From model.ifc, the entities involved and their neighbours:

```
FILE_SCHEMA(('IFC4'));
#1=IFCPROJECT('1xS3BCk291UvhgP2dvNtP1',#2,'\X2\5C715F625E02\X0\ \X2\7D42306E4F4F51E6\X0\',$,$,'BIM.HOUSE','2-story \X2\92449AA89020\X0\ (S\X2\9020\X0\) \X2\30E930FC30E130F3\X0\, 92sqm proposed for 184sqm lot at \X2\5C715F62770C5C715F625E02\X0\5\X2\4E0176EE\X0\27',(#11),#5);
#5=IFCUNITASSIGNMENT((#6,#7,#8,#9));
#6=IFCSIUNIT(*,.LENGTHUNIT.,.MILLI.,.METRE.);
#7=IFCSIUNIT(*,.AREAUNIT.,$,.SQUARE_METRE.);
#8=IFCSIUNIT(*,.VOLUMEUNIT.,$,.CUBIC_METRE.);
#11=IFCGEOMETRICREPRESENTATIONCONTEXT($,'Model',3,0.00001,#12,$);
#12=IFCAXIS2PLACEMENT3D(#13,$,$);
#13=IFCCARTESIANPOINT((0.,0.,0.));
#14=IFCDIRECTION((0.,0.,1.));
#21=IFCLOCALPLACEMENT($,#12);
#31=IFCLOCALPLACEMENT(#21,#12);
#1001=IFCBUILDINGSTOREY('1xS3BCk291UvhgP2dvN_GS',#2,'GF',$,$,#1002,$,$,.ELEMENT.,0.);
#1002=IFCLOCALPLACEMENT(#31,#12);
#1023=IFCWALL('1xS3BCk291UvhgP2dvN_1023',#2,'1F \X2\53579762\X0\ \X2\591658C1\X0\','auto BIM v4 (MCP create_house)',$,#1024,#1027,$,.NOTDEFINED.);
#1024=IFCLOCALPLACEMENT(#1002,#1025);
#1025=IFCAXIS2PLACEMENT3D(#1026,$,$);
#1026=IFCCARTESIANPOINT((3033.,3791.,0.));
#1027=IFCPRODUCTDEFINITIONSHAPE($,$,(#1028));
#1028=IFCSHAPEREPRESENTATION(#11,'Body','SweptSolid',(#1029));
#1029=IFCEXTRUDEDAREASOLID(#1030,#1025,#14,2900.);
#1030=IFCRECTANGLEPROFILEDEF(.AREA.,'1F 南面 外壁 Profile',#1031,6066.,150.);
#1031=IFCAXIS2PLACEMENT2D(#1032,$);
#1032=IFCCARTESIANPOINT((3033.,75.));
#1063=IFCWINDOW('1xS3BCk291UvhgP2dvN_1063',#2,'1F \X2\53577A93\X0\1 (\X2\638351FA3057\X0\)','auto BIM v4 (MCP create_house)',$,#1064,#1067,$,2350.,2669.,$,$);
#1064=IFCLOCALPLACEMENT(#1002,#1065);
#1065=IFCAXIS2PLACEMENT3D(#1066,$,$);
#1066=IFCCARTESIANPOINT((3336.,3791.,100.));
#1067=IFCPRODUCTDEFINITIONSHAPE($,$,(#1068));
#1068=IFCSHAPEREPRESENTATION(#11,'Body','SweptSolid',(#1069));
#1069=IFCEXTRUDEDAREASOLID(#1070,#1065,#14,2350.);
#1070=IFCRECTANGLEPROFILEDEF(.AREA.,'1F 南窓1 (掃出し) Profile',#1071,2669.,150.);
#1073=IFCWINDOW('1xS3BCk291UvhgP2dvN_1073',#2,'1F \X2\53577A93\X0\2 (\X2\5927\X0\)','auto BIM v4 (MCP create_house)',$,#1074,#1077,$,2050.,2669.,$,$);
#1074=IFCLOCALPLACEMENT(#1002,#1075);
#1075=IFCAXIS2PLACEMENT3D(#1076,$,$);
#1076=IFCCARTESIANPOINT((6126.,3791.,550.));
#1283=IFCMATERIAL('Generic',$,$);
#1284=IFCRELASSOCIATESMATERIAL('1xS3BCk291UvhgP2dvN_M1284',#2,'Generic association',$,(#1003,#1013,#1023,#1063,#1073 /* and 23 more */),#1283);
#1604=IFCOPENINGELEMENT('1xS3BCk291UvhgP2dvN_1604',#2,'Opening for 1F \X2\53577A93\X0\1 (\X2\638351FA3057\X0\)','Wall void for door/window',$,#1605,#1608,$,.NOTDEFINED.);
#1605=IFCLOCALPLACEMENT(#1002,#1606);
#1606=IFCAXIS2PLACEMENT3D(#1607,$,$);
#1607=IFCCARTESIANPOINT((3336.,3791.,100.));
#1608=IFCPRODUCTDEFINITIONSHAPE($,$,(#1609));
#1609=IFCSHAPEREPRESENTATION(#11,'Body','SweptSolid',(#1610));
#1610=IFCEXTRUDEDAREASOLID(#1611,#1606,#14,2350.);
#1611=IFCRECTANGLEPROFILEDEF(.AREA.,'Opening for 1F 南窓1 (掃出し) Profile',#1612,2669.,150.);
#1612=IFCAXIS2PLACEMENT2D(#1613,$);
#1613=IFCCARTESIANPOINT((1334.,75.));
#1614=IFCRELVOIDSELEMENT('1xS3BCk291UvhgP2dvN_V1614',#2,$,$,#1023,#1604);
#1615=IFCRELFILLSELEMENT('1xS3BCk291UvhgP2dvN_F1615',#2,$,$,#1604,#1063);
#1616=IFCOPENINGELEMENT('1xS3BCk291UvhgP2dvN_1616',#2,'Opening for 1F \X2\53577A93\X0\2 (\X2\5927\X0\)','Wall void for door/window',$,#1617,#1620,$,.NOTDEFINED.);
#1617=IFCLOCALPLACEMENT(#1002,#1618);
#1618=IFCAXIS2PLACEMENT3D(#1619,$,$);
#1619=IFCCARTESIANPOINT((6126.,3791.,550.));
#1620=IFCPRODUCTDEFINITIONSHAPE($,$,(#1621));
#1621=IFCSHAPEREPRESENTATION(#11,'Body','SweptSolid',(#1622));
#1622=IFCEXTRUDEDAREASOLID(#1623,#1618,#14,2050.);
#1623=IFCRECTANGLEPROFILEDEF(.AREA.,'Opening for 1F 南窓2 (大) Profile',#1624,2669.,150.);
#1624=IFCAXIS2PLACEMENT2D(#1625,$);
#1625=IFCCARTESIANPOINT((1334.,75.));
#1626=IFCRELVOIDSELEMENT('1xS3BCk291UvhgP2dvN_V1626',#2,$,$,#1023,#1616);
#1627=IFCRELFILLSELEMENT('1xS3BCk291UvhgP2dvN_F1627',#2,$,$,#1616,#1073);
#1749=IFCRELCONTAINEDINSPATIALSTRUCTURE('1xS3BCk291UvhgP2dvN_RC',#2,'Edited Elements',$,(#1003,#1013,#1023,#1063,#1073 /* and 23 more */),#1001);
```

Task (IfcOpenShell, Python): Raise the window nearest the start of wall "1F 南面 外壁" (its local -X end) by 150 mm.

```python
import numpy as np
import ifcopenshell
import ifcopenshell.api.geometry
import ifcopenshell.util.placement
import ifcopenshell.util.unit

model = ifcopenshell.open("model.ifc")
unit_scale = ifcopenshell.util.unit.calculate_unit_scale(model)

window = model.by_guid("1xS3BCk291UvhgP2dvN_1063")
opening = window.FillsVoids[0].RelatingOpeningElement
dz = 150.0

shift = np.array([0.0, 0.0, dz])
# The window is not placed relative to its opening, so move both.
for product in (opening, window):
    matrix = ifcopenshell.util.placement.get_local_placement(product.ObjectPlacement)
    matrix[:3, 3] += shift
    ifcopenshell.api.geometry.edit_object_placement(model, product=product, matrix=matrix, is_si=False)

print(f"moved by {dz * unit_scale:+.3f} m")

model.write("model_updated.ifc")
```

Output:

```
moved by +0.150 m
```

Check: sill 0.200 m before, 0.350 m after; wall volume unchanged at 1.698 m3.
